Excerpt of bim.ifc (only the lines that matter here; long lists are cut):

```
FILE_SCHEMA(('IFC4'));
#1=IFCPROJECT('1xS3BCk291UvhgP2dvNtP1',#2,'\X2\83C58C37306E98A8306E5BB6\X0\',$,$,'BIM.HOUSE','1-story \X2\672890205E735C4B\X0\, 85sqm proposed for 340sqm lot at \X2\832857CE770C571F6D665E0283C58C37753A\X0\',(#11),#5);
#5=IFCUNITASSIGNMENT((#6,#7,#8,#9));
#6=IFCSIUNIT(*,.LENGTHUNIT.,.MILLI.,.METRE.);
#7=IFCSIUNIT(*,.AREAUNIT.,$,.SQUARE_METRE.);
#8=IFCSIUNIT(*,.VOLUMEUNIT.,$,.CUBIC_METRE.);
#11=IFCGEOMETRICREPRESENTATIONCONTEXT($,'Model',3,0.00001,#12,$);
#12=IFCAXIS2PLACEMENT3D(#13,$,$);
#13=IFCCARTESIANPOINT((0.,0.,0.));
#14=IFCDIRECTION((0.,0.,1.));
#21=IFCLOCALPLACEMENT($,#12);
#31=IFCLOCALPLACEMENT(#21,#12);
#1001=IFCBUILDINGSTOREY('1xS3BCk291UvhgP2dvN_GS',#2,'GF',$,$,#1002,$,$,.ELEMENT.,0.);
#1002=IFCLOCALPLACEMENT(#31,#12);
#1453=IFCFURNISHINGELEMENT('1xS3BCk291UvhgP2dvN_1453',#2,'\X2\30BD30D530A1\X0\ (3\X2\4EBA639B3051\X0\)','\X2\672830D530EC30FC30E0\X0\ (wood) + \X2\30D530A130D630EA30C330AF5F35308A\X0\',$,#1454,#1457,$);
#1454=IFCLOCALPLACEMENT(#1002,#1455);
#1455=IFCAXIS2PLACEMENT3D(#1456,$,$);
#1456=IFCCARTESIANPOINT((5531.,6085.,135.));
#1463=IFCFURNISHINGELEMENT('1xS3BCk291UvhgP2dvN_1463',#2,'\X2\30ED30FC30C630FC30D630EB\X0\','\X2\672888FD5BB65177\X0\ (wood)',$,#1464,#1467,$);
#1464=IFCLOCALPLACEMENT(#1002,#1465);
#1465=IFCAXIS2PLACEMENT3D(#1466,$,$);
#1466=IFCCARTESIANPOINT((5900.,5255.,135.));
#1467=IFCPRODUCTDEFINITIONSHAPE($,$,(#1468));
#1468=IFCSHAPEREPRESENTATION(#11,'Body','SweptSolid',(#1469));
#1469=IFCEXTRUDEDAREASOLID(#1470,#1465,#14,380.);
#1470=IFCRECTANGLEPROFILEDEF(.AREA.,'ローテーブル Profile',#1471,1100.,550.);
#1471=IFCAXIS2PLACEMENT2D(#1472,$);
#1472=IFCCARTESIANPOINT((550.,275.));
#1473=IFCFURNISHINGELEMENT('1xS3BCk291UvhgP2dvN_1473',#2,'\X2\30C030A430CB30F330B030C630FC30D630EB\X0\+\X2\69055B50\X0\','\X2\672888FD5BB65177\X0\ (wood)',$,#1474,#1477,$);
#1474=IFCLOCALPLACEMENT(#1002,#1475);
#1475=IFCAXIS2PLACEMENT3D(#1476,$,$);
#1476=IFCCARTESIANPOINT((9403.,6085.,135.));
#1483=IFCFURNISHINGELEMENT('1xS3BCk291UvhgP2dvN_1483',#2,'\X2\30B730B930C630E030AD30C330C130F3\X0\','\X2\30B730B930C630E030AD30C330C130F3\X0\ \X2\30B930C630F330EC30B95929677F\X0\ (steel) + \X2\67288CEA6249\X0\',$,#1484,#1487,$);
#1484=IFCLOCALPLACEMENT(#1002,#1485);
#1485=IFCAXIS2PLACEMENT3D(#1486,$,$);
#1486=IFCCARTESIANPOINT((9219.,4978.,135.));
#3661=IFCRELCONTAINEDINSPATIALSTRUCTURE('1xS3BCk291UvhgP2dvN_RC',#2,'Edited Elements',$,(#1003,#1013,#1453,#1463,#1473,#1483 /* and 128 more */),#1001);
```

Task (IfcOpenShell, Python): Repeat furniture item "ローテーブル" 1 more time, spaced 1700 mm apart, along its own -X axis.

```python
import ifcopenshell
import ifcopenshell.api.geometry
import ifcopenshell.api.root
import ifcopenshell.util.element
import ifcopenshell.util.placement
import ifcopenshell.util.unit

model = ifcopenshell.open("bim.ifc")
unit_scale = ifcopenshell.util.unit.calculate_unit_scale(model)


def reuse_history(source, copy):
    """copy_class also copies each property set's owner history, people and application; keep the originals."""
    for rel in copy.IsDefinedBy:
        if rel.is_a("IfcRelDefinesByProperties") and (history := rel.RelatingPropertyDefinition.OwnerHistory):
            rel.RelatingPropertyDefinition.OwnerHistory = source.OwnerHistory
            ifcopenshell.util.element.remove_deep2(model, history)


source = model.by_id(1463)
base = ifcopenshell.util.placement.get_local_placement(source.ObjectPlacement)
step = -base[:3, 0] * 1.7 / unit_scale

for i in range(1, 2):
    copy = ifcopenshell.api.root.copy_class(model, product=source)
    copy.Representation = ifcopenshell.util.element.copy_deep(
        model, source.Representation, exclude=["IfcGeometricRepresentationContext", "IfcRepresentationMap"]
    )
    reuse_history(source, copy)
    matrix = base.copy()
    matrix[:3, 3] += i * step
    print("added at", matrix[:3, 3].round(3) + 0.0)
    ifcopenshell.api.geometry.edit_object_placement(model, product=copy, matrix=matrix, is_si=False)

model.write("bim-out.ifc")
```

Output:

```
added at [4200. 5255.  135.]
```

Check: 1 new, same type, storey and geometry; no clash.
